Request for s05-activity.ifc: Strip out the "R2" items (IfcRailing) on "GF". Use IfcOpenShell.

First a look at what the model holds.

```python
import ifcopenshell
import ifcopenshell.util.element

model = ifcopenshell.open("s05-activity.ifc")
print(model.schema)
storey = next(s for s in model.by_type("IfcBuildingStorey") if s.Name == "GF")
railings = [e for e in ifcopenshell.util.element.get_decomposition(storey) if e.is_a("IfcRailing")]
seen = {}
for e in railings:
    element_type = ifcopenshell.util.element.get_type(e)
    name = element_type.Name if element_type not in (None, e) else None
    seen[name] = seen.get(name, 0) + 1
for name, count in sorted(seen.items(), key=str):
    print(count, "x", name)
```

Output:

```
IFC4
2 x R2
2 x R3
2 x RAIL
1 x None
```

```python
import ifcopenshell
import ifcopenshell.api.root
import ifcopenshell.util.element

model = ifcopenshell.open("s05-activity.ifc")

storey = next(s for s in model.by_type("IfcBuildingStorey") if s.Name == "GF")
railings = [e for e in ifcopenshell.util.element.get_decomposition(storey) if e.is_a("IfcRailing")]
targets = [e for e in railings if (t := ifcopenshell.util.element.get_type(e)) not in (None, e) and t.Name == "R2"]

for e in targets:
    ifcopenshell.api.root.remove_product(model, product=e)
print(len(targets), "removed")

model.write("s05-activity_edited.ifc")
```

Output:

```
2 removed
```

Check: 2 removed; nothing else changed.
